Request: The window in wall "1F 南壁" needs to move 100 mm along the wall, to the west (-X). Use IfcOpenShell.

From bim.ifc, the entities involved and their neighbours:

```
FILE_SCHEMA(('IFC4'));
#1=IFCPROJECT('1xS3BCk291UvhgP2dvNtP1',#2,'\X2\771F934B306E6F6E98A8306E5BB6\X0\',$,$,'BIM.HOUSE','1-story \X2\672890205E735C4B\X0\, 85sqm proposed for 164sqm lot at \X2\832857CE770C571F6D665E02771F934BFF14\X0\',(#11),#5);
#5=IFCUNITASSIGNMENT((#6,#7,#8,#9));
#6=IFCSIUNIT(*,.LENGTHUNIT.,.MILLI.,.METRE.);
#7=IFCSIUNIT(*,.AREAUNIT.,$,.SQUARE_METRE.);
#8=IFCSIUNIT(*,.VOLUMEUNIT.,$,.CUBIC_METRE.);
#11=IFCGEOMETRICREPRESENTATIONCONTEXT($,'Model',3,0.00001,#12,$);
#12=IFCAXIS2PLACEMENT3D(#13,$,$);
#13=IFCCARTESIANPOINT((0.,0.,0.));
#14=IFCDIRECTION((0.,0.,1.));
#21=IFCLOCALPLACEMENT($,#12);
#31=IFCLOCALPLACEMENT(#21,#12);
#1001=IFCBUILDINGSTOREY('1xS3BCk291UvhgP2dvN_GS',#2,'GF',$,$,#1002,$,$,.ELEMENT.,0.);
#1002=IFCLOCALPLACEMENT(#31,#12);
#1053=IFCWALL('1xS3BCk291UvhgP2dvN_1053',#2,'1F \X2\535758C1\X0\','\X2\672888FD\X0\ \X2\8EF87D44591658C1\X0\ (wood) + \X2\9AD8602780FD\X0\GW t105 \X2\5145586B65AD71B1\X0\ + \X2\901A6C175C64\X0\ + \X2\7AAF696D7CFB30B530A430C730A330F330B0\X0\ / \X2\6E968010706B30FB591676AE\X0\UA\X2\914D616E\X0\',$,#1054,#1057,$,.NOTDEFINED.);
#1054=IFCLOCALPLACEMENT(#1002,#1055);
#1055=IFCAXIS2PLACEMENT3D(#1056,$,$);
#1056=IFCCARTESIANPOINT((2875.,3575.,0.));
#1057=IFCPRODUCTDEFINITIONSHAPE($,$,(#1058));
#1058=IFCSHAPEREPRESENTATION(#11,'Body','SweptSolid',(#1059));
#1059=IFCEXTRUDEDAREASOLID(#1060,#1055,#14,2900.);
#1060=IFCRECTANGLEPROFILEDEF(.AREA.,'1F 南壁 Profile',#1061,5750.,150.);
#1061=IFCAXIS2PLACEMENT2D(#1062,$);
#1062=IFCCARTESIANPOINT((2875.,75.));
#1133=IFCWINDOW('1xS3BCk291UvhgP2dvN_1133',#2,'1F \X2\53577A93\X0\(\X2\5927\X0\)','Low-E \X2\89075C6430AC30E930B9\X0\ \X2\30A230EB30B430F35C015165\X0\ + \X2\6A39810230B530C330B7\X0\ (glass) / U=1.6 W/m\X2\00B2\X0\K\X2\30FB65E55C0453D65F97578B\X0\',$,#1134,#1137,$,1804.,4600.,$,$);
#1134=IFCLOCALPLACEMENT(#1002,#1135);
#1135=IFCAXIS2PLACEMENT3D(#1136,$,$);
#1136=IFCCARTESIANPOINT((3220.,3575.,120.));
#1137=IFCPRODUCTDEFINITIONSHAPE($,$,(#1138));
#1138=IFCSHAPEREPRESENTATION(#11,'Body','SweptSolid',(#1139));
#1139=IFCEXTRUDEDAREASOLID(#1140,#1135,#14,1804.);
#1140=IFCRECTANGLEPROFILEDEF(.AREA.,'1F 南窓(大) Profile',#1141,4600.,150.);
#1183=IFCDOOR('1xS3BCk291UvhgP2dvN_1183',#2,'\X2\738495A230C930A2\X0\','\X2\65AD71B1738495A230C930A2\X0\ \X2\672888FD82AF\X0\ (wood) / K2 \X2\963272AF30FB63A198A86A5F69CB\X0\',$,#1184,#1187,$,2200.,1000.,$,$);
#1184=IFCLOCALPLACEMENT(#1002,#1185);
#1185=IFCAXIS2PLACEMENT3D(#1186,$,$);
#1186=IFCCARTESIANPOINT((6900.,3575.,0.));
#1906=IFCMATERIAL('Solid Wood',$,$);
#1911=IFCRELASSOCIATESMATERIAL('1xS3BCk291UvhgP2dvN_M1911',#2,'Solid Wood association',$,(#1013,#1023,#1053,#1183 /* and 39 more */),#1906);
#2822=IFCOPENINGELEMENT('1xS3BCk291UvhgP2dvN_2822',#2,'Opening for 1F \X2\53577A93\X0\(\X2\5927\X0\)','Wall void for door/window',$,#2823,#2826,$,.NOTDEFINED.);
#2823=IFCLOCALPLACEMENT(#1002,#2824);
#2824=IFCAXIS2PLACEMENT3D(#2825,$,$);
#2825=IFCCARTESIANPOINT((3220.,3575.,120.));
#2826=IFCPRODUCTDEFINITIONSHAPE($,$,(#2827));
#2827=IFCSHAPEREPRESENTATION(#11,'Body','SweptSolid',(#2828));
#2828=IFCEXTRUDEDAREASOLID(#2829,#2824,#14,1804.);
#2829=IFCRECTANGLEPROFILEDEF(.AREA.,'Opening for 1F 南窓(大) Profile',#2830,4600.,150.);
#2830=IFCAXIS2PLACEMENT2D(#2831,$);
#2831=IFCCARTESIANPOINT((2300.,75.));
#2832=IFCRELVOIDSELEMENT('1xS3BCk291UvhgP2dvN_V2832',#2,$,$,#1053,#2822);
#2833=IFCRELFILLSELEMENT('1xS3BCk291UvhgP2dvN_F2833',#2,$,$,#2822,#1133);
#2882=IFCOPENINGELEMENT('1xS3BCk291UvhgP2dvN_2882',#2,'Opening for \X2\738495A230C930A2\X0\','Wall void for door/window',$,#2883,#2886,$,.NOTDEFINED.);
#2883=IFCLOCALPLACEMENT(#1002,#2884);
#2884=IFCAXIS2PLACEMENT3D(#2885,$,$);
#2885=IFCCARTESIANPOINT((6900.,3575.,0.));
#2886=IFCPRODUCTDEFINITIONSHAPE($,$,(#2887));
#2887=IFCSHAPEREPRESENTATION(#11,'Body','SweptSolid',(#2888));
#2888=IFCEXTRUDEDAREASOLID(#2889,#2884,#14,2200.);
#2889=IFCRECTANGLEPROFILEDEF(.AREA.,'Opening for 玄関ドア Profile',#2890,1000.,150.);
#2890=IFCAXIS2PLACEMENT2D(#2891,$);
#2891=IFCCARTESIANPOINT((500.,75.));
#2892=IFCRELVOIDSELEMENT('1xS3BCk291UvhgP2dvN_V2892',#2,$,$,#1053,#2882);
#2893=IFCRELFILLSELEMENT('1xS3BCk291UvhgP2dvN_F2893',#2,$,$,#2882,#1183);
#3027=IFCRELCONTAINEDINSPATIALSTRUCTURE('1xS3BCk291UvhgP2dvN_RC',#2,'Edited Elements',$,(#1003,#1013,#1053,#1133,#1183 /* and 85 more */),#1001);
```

```python
import ifcopenshell
import ifcopenshell.api.geometry
import ifcopenshell.util.placement
import ifcopenshell.util.unit

model = ifcopenshell.open("bim.ifc")
unit_scale = ifcopenshell.util.unit.calculate_unit_scale(model)

window = model.by_guid("1xS3BCk291UvhgP2dvN_1133")
opening = window.FillsVoids[0].RelatingOpeningElement
wall = opening.VoidsElements[0].RelatingBuildingElement

wall_matrix = ifcopenshell.util.placement.get_local_placement(wall.ObjectPlacement)
shift = wall_matrix[:3, 0] * -0.1 / unit_scale
before = ifcopenshell.util.placement.get_local_placement(window.ObjectPlacement)[:3, 3].copy()

# The window is not placed relative to its opening, so move both.
for product in (opening, window):
    matrix = ifcopenshell.util.placement.get_local_placement(product.ObjectPlacement)
    matrix[:3, 3] += shift
    ifcopenshell.api.geometry.edit_object_placement(model, product=product, matrix=matrix, is_si=False)

after = ifcopenshell.util.placement.get_local_placement(window.ObjectPlacement)[:3, 3]
print("window moved by", (after - before).round(3) + 0.0)

model.write("bim_rev.ifc")
```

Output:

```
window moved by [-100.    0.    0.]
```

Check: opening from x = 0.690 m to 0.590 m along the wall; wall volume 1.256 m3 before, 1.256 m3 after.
